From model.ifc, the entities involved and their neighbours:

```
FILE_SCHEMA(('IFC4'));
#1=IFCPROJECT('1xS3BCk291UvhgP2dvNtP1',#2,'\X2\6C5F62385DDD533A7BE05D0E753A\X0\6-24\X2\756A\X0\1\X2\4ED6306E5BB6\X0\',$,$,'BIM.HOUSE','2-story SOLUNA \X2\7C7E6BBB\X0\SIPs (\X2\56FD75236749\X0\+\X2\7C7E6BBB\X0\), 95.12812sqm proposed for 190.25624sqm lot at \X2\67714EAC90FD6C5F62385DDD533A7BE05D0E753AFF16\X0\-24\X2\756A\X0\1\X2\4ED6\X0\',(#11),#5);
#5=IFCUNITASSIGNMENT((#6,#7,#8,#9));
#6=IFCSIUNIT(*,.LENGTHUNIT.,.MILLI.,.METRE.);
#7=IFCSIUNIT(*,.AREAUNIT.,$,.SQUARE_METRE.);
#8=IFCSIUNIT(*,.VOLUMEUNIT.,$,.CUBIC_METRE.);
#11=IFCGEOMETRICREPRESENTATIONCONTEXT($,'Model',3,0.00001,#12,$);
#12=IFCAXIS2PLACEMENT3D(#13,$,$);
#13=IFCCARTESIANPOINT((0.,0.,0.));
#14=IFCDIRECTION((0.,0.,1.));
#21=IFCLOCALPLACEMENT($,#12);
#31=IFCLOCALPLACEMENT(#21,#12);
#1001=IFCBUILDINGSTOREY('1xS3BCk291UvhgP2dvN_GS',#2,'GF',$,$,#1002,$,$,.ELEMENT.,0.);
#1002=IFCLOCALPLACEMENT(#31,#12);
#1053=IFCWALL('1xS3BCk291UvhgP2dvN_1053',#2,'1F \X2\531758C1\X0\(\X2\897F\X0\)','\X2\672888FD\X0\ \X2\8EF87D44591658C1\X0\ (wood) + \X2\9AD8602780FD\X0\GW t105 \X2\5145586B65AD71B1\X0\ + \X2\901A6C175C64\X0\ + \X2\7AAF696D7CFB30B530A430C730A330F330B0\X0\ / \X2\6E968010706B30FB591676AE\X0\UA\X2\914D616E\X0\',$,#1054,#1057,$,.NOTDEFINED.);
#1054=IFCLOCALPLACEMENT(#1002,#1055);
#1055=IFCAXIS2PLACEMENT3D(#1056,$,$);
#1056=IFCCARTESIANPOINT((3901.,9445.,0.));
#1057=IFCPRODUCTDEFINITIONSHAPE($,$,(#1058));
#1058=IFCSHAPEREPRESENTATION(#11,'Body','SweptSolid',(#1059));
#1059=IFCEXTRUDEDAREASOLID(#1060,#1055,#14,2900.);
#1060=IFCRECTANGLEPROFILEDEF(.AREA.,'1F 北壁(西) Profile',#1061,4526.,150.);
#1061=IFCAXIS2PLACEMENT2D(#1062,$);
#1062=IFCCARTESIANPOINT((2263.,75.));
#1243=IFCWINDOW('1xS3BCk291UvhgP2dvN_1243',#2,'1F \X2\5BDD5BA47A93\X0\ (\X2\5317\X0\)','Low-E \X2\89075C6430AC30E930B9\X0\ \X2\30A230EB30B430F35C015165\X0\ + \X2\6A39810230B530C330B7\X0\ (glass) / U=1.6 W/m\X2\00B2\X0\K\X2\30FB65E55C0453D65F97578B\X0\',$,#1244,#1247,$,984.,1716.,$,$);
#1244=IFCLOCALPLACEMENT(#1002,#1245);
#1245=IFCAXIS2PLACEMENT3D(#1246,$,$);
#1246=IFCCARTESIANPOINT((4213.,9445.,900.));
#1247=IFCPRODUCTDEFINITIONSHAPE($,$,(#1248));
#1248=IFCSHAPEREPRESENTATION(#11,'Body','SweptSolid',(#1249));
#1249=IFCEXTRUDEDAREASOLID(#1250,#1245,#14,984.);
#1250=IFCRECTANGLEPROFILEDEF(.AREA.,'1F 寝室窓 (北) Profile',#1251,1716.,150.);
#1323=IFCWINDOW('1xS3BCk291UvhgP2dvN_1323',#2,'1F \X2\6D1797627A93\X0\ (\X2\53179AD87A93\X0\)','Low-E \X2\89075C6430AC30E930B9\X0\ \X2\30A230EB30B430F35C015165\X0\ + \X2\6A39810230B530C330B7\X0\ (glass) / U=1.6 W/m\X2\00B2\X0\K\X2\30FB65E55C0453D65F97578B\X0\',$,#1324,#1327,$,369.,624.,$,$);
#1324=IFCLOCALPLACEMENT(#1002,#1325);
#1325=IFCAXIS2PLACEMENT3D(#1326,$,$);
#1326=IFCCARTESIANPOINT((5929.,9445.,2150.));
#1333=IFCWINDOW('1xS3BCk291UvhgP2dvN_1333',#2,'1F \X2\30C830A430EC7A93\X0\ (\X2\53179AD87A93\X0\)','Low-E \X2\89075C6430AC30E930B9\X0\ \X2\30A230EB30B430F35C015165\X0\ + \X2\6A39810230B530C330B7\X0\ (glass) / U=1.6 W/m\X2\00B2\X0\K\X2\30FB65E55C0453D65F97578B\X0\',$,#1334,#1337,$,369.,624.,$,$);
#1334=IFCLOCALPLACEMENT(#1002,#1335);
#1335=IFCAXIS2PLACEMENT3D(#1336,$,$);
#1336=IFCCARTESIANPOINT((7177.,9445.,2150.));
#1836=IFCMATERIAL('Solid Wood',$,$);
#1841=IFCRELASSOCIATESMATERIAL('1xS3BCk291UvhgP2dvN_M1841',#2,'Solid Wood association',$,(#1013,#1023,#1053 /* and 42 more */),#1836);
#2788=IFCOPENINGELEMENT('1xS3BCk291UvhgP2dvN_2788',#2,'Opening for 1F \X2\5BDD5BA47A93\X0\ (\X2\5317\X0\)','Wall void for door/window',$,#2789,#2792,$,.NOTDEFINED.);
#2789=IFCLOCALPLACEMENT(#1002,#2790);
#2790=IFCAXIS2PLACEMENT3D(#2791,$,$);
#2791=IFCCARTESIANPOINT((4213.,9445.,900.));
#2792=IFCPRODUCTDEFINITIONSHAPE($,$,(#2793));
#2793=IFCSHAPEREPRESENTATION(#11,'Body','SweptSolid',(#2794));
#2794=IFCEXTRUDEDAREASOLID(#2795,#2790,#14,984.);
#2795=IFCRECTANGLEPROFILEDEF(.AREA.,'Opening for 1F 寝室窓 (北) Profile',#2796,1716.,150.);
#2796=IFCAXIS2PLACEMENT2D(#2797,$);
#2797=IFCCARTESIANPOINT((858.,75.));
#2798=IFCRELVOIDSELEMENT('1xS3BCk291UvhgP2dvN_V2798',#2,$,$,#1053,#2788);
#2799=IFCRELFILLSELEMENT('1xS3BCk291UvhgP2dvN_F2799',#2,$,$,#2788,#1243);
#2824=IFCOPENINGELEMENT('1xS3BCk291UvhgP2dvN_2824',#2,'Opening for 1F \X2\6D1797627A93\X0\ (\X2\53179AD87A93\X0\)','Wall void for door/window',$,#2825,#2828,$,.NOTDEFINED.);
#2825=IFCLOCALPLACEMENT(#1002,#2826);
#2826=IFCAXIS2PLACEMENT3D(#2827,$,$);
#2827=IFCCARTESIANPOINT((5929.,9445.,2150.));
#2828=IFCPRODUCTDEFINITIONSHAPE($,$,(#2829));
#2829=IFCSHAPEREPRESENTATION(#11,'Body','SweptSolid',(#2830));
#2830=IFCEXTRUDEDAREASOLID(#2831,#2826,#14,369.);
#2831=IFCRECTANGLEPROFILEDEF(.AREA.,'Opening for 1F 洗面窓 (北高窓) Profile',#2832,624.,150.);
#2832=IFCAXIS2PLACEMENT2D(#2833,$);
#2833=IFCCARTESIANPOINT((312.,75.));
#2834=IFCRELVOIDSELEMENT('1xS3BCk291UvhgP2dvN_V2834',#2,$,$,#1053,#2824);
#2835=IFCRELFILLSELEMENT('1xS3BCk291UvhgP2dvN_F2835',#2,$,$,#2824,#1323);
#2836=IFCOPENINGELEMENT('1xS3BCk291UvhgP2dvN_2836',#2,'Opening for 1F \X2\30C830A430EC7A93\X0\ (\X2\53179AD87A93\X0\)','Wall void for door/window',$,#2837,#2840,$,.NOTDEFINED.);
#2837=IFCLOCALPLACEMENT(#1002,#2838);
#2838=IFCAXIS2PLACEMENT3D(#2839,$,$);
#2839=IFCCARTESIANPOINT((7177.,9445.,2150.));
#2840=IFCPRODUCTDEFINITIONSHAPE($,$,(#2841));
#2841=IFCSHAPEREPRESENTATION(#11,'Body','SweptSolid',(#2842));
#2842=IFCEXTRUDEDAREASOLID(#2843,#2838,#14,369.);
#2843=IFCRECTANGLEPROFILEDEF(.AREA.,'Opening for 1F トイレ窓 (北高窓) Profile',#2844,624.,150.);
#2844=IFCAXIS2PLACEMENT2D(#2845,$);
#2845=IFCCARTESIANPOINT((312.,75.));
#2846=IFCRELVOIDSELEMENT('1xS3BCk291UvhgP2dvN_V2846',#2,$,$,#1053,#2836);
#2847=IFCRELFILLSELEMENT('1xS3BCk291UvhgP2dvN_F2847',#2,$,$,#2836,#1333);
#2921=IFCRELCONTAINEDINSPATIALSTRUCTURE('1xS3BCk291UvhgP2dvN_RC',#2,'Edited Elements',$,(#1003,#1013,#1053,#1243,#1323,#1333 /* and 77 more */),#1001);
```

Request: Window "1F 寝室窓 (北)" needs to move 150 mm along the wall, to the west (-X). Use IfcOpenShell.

```python
import ifcopenshell
import ifcopenshell.api.geometry
import ifcopenshell.util.placement

model = ifcopenshell.open("model.ifc")

window = model.by_guid("1xS3BCk291UvhgP2dvN_1243")
opening = window.FillsVoids[0].RelatingOpeningElement
wall = opening.VoidsElements[0].RelatingBuildingElement

wall_matrix = ifcopenshell.util.placement.get_local_placement(wall.ObjectPlacement)
shift = wall_matrix[:3, 0] * -150.0
before = ifcopenshell.util.placement.get_local_placement(window.ObjectPlacement)[:3, 3].copy()

# The window is not placed relative to its opening, so move both.
for product in (opening, window):
    matrix = ifcopenshell.util.placement.get_local_placement(product.ObjectPlacement)
    matrix[:3, 3] += shift
    ifcopenshell.api.geometry.edit_object_placement(model, product=product, matrix=matrix, is_si=False)

after = ifcopenshell.util.placement.get_local_placement(window.ObjectPlacement)[:3, 3]
print("window moved by", (after - before).round(3) + 0.0)

model.write("model_edited.ifc")
```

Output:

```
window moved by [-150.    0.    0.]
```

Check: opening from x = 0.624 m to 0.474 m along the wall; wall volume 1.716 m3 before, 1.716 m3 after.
